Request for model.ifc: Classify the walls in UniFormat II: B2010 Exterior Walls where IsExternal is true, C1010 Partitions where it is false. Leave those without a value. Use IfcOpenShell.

First a look at what the model holds.

```python
import ifcopenshell
import ifcopenshell.util.element

model = ifcopenshell.open("model.ifc")
print(model.schema)
print("classifications:", [c.Name for c in model.by_type("IfcClassification")])
values = [ifcopenshell.util.element.get_pset(e, "Pset_WallCommon", "IsExternal") for e in model.by_type("IfcWall")]
for value in (True, False, None):
    print("IsExternal", value, values.count(value))
```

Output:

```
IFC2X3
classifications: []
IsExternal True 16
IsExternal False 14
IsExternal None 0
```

```python
import ifcopenshell
import ifcopenshell.api.classification
import ifcopenshell.util.element

model = ifcopenshell.open("model.ifc")

# IFC2X3 requires Source and Edition and has no link from the project to the system.
system = model.create_entity("IfcClassification", Source="ASTM", Edition="E1557", Name="UniFormat II")

walls = model.by_type("IfcWall")
external = {e: ifcopenshell.util.element.get_pset(e, "Pset_WallCommon", "IsExternal") for e in walls}
for flag, code, name in ((True, "B2010", "Exterior Walls"), (False, "C1010", "Partitions")):
    products = [e for e in walls if external[e] is flag]
    ifcopenshell.api.classification.add_reference(
        model, products=products, classification=system, identification=code, name=name
    )
    print(code, len(products))

model.write("model_edited.ifc")
```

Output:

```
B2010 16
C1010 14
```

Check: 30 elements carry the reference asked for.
